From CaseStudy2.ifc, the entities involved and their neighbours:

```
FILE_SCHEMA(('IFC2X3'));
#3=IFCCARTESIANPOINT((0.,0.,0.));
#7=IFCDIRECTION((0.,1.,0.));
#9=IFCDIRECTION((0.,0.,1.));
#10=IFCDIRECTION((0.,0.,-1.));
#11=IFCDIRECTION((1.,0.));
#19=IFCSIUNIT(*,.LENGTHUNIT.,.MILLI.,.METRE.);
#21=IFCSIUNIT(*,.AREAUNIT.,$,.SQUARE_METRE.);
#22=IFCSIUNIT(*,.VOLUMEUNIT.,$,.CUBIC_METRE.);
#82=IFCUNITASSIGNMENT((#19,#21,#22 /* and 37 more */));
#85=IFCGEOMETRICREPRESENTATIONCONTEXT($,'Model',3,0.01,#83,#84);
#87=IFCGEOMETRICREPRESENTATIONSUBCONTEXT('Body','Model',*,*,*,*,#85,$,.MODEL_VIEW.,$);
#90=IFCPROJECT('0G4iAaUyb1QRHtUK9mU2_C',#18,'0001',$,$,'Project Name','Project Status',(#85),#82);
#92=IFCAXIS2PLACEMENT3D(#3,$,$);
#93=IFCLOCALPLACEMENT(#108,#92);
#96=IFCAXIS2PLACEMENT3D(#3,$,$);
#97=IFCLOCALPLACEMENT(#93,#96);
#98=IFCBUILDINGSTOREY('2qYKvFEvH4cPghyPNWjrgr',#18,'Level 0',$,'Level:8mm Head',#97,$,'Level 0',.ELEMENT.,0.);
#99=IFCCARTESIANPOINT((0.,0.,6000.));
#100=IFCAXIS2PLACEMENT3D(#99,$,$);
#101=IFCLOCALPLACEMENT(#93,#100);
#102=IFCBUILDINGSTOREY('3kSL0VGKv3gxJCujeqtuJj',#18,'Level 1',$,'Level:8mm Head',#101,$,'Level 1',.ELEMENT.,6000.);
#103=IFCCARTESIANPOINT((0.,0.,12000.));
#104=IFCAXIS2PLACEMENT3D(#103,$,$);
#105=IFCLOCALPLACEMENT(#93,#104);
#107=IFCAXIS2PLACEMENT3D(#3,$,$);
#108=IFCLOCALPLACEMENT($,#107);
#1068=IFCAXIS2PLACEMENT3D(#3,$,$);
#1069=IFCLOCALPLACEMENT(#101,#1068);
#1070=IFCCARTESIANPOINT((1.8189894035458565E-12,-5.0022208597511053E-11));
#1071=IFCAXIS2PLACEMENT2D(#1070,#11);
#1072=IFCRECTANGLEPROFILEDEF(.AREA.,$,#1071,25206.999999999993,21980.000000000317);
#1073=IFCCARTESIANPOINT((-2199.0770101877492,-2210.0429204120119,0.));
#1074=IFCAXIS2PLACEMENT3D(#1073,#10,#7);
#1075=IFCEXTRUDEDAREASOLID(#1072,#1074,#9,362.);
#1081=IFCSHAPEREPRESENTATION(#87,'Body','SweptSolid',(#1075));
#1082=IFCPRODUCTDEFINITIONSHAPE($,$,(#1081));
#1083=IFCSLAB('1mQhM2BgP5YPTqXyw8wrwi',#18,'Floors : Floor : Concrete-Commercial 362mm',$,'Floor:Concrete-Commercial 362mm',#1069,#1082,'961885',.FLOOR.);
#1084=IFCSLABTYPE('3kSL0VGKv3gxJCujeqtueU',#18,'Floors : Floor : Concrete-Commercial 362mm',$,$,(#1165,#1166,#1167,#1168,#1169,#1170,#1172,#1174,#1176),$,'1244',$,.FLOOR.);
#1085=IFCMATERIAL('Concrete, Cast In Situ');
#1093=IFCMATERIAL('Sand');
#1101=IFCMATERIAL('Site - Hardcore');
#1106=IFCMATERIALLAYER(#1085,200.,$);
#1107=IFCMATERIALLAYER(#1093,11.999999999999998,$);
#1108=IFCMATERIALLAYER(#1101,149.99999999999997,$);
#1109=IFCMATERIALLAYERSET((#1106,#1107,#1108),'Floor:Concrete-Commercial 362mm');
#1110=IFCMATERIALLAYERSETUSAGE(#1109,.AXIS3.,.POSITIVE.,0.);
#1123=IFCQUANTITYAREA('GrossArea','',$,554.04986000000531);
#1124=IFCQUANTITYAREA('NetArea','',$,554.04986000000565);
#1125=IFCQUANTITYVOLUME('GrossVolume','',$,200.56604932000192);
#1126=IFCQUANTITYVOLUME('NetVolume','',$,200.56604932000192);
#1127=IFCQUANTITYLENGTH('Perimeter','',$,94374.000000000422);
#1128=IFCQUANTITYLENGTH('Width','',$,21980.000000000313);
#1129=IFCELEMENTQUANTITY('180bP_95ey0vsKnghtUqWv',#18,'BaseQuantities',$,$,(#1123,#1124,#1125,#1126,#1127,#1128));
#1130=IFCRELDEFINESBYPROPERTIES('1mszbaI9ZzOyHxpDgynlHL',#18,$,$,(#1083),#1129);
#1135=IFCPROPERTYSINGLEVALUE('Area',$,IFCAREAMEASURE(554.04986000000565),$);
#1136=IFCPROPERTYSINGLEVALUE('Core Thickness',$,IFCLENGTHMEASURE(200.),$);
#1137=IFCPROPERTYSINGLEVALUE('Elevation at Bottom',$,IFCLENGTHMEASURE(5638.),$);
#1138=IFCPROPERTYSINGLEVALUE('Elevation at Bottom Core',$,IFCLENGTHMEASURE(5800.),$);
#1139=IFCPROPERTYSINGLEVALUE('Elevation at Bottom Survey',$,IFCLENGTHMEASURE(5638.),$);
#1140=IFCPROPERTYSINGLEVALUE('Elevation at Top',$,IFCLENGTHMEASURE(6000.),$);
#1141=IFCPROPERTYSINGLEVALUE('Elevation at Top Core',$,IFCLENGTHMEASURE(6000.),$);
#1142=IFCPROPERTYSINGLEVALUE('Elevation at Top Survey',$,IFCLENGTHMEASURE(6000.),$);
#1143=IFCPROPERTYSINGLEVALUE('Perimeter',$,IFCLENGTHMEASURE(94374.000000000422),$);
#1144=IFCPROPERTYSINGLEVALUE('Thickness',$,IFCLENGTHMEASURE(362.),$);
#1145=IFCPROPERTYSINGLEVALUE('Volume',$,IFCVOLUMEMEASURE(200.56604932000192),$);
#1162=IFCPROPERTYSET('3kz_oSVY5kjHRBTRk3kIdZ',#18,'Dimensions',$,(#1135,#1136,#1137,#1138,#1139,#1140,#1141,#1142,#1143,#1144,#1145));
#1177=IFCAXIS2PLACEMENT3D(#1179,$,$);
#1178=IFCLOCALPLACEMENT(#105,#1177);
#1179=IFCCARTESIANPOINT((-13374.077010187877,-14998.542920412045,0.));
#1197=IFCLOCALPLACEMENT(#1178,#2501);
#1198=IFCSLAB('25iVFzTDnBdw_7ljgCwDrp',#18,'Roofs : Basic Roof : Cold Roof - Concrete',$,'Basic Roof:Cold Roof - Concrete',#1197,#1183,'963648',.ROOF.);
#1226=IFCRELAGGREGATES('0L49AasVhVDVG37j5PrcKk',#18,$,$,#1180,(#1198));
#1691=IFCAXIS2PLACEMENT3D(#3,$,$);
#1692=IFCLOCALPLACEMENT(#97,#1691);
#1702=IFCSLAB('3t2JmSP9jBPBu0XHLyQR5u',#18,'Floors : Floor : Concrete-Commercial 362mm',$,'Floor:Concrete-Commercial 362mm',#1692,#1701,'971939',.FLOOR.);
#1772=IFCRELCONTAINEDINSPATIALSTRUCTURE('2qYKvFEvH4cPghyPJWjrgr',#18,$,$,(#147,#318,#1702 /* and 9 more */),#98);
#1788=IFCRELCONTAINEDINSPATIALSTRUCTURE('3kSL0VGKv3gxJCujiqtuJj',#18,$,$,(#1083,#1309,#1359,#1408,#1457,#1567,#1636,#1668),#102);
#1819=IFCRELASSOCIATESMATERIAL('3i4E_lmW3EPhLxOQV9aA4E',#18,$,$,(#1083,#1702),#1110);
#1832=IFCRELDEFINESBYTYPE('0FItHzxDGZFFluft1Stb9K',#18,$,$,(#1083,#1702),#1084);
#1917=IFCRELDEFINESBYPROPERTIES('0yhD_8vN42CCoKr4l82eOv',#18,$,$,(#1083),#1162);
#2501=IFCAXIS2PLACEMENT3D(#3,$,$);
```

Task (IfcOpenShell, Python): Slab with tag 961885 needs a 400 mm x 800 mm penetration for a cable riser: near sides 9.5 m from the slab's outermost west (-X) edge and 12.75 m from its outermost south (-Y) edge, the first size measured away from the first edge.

```python
import numpy as np
import ifcopenshell
import ifcopenshell.api.feature
import ifcopenshell.api.geometry
import ifcopenshell.api.pset
import ifcopenshell.api.root
import ifcopenshell.geom
import ifcopenshell.util.element
import ifcopenshell.util.placement
import ifcopenshell.util.representation
import ifcopenshell.util.shape
import ifcopenshell.util.unit

model = ifcopenshell.open("CaseStudy2.ifc")
unit_scale = ifcopenshell.util.unit.calculate_unit_scale(model)
area_scale = ifcopenshell.util.unit.calculate_unit_scale(model, "AREAUNIT")
volume_scale = ifcopenshell.util.unit.calculate_unit_scale(model, "VOLUMEUNIT")
settings = ifcopenshell.geom.settings()


def volume(element):
    """Net volume in cubic metres, openings subtracted."""
    shape = ifcopenshell.geom.create_shape(settings, element)
    return ifcopenshell.util.shape.get_volume(shape.geometry)


slab = model.by_guid("1mQhM2BgP5YPTqXyw8wrwi")
before = volume(slab)

# Extent in the slab's own axes, in metres. The edges named are its -X and -Y sides.
slab_shape = ifcopenshell.geom.create_shape(settings, slab)
vertices = ifcopenshell.util.shape.get_vertices(slab_shape.geometry)
x_min, y_min, bottom = vertices.min(axis=0)
top = vertices[:, 2].max()

opening = ifcopenshell.api.root.create_entity(model, ifc_class="IfcOpeningElement", name="Cable riser opening")
context = ifcopenshell.util.representation.get_context(model, "Model", "Body", "MODEL_VIEW")
width, depth = 0.4, 0.8
outline = [(0.0, 0.0), (width, 0.0), (width, depth), (0.0, depth), (0.0, 0.0)]
# Overshoot both faces by 50 mm so the cut is clean.
shape = ifcopenshell.api.geometry.add_slab_representation(
    model, context=context, depth=top - bottom + 0.1, polyline=outline
)
ifcopenshell.api.geometry.assign_representation(model, product=opening, representation=shape)

matrix = ifcopenshell.util.placement.get_local_placement(slab.ObjectPlacement)
matrix[:, 3] = matrix @ np.append(np.array([x_min + 9.5, y_min + 12.75, bottom - 0.05]) / unit_scale, 1.0)
ifcopenshell.api.geometry.edit_object_placement(model, product=opening, matrix=matrix, is_si=False)
ifcopenshell.api.feature.add_feature(model, feature=opening, element=slab)

after = volume(slab)

# Update the slab's stored quantities.
qto = model.by_id(ifcopenshell.util.element.get_pset(slab, "BaseQuantities", should_inherit=False)["id"])
ifcopenshell.api.pset.edit_qto(model, qto=qto, properties={
    "NetArea": after / (top - bottom) / area_scale,
    "NetVolume": after / volume_scale,
})
pset = model.by_id(ifcopenshell.util.element.get_pset(slab, "Dimensions", should_inherit=False)["id"])
ifcopenshell.api.pset.edit_pset(model, pset=pset, properties={
    "Area": model.create_entity("IfcAreaMeasure", after / (top - bottom) / area_scale),
    "Volume": model.create_entity("IfcVolumeMeasure", after / volume_scale),
})

print(f"slab volume {before:.3f} -> {after:.3f} m3")

model.write("CaseStudy2-out.ifc")
```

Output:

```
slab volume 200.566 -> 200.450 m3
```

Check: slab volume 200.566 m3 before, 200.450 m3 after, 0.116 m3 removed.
